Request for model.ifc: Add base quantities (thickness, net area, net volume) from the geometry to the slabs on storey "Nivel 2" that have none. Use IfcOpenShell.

First a look at what the model holds.

```python
import ifcopenshell
import ifcopenshell.util.element
import ifcopenshell.util.unit

model = ifcopenshell.open("model.ifc")
print(model.schema)
for unit_type in ("LENGTHUNIT", "AREAUNIT", "VOLUMEUNIT"):
    print(unit_type, ifcopenshell.util.unit.calculate_unit_scale(model, unit_type))
storey = next(s for s in model.by_type("IfcBuildingStorey") if s.Name == "Nivel 2")
slabs = [e for e in ifcopenshell.util.element.get_decomposition(storey) if e.is_a("IfcSlab")]
for e in sorted(slabs, key=lambda e: e.id()):
    print(e.id(), e.is_a(), e.Name, list(ifcopenshell.util.element.get_psets(e, qtos_only=True)), sep=" | ")
```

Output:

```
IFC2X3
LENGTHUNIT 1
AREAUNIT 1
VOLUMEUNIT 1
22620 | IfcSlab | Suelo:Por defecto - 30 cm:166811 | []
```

```python
import ifcopenshell
import ifcopenshell.api.pset
import ifcopenshell.geom
import ifcopenshell.util.element
import ifcopenshell.util.shape
import ifcopenshell.util.unit

model = ifcopenshell.open("model.ifc")
unit_scale = ifcopenshell.util.unit.calculate_unit_scale(model)
area_scale = ifcopenshell.util.unit.calculate_unit_scale(model, "AREAUNIT")
volume_scale = ifcopenshell.util.unit.calculate_unit_scale(model, "VOLUMEUNIT")
settings = ifcopenshell.geom.settings()

storey = next(s for s in model.by_type("IfcBuildingStorey") if s.Name == "Nivel 2")
slabs = [e for e in ifcopenshell.util.element.get_decomposition(storey) if e.is_a("IfcSlab")]

for e in sorted(slabs, key=lambda e: e.id()):
    if ifcopenshell.util.element.get_psets(e, qtos_only=True, should_inherit=False):
        continue
    # Geometry comes back in metres, in the element's own axes.
    shape = ifcopenshell.geom.create_shape(settings, e)
    values = {
        "Width": ifcopenshell.util.shape.get_z(shape.geometry) / unit_scale,
        "NetArea": ifcopenshell.util.shape.get_footprint_area(shape.geometry) / area_scale,
        "NetVolume": ifcopenshell.util.shape.get_volume(shape.geometry) / volume_scale,
    }
    qto = ifcopenshell.api.pset.add_qto(model, product=e, name="BaseQuantities")
    ifcopenshell.api.pset.edit_qto(model, qto=qto, properties=values)
    print(e.id(), {k: round(v, 3) for k, v in values.items()})

model.write("model_rev.ifc")
```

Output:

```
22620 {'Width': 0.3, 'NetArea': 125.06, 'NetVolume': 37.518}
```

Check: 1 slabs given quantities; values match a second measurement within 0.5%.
